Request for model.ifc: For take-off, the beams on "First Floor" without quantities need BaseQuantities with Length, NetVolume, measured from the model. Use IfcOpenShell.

First a look at what the model holds.

```python
import ifcopenshell
import ifcopenshell.util.element
import ifcopenshell.util.unit

model = ifcopenshell.open("model.ifc")
print(model.schema)
for unit_type in ("LENGTHUNIT", "AREAUNIT", "VOLUMEUNIT"):
    print(unit_type, ifcopenshell.util.unit.calculate_unit_scale(model, unit_type))
storey = next(s for s in model.by_type("IfcBuildingStorey") if s.Name == "First Floor")
beams = [e for e in ifcopenshell.util.element.get_decomposition(storey) if e.is_a("IfcBeam")]
for e in sorted(beams, key=lambda e: e.id()):
    print(e.id(), e.is_a(), e.Name, list(ifcopenshell.util.element.get_psets(e, qtos_only=True)), sep=" | ")
```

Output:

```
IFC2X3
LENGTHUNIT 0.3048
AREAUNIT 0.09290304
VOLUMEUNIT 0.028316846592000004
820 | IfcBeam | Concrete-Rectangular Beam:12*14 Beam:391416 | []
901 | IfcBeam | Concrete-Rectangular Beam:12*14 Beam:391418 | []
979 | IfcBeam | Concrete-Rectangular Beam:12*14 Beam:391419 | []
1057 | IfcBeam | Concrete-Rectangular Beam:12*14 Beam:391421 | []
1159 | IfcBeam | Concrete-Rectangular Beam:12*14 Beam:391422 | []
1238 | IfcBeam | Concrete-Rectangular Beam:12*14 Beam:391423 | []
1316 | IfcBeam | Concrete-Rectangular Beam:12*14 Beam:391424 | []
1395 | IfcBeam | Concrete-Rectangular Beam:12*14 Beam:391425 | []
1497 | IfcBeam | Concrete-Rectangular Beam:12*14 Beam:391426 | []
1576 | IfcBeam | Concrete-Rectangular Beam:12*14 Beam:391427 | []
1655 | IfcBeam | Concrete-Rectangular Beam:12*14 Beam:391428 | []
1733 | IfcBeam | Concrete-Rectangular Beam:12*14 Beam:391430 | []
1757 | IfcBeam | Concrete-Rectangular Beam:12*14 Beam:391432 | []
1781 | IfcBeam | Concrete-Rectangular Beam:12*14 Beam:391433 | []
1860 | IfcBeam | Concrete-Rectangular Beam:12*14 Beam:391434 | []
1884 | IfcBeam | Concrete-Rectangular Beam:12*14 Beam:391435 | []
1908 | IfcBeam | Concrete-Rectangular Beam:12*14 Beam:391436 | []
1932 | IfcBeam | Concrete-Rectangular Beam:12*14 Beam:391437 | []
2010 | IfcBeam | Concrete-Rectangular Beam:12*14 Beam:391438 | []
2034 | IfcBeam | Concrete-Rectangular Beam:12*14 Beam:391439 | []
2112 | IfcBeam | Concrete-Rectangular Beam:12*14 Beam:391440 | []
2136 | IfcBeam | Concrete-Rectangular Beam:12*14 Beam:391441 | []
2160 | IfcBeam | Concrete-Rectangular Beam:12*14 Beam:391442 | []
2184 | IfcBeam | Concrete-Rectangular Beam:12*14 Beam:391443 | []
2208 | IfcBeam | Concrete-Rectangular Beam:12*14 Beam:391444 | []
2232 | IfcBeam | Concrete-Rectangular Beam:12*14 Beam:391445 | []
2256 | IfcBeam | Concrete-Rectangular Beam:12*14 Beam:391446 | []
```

```python
import ifcopenshell
import ifcopenshell.api.pset
import ifcopenshell.geom
import ifcopenshell.util.element
import ifcopenshell.util.shape
import ifcopenshell.util.unit

model = ifcopenshell.open("model.ifc")
unit_scale = ifcopenshell.util.unit.calculate_unit_scale(model)
volume_scale = ifcopenshell.util.unit.calculate_unit_scale(model, "VOLUMEUNIT")
settings = ifcopenshell.geom.settings()

storey = next(s for s in model.by_type("IfcBuildingStorey") if s.Name == "First Floor")
beams = [e for e in ifcopenshell.util.element.get_decomposition(storey) if e.is_a("IfcBeam")]

for e in sorted(beams, key=lambda e: e.id()):
    if ifcopenshell.util.element.get_psets(e, qtos_only=True, should_inherit=False):
        continue
    # Geometry comes back in metres, in the element's own axes.
    shape = ifcopenshell.geom.create_shape(settings, e)
    values = {
        "Length": ifcopenshell.util.shape.get_max_xyz(shape.geometry) / unit_scale,
        "NetVolume": ifcopenshell.util.shape.get_volume(shape.geometry) / volume_scale,
    }
    qto = ifcopenshell.api.pset.add_qto(model, product=e, name="BaseQuantities")
    ifcopenshell.api.pset.edit_qto(model, qto=qto, properties=values)
    print(e.id(), {k: round(v, 3) for k, v in values.items()})

model.write("model_rev.ifc")
```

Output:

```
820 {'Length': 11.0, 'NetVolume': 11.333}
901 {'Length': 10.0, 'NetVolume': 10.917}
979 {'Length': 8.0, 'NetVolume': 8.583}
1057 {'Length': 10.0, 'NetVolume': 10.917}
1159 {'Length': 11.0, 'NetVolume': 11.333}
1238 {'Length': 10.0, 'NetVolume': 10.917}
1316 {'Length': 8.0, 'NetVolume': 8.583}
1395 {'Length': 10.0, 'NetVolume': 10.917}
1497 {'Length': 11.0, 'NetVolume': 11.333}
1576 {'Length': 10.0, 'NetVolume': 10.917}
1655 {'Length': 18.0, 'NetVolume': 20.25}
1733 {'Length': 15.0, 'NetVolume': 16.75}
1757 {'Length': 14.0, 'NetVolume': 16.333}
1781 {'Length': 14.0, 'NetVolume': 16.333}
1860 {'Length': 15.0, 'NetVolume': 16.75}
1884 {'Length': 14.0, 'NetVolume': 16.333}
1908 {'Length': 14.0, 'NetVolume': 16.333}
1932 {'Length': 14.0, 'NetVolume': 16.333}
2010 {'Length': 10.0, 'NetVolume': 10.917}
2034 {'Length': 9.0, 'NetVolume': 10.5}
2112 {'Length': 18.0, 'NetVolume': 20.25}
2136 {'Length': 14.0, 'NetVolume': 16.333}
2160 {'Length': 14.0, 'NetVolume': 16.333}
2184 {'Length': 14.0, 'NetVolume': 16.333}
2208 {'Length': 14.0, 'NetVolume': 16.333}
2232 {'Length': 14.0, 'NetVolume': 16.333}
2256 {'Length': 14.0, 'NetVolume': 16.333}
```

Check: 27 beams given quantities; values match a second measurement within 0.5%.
